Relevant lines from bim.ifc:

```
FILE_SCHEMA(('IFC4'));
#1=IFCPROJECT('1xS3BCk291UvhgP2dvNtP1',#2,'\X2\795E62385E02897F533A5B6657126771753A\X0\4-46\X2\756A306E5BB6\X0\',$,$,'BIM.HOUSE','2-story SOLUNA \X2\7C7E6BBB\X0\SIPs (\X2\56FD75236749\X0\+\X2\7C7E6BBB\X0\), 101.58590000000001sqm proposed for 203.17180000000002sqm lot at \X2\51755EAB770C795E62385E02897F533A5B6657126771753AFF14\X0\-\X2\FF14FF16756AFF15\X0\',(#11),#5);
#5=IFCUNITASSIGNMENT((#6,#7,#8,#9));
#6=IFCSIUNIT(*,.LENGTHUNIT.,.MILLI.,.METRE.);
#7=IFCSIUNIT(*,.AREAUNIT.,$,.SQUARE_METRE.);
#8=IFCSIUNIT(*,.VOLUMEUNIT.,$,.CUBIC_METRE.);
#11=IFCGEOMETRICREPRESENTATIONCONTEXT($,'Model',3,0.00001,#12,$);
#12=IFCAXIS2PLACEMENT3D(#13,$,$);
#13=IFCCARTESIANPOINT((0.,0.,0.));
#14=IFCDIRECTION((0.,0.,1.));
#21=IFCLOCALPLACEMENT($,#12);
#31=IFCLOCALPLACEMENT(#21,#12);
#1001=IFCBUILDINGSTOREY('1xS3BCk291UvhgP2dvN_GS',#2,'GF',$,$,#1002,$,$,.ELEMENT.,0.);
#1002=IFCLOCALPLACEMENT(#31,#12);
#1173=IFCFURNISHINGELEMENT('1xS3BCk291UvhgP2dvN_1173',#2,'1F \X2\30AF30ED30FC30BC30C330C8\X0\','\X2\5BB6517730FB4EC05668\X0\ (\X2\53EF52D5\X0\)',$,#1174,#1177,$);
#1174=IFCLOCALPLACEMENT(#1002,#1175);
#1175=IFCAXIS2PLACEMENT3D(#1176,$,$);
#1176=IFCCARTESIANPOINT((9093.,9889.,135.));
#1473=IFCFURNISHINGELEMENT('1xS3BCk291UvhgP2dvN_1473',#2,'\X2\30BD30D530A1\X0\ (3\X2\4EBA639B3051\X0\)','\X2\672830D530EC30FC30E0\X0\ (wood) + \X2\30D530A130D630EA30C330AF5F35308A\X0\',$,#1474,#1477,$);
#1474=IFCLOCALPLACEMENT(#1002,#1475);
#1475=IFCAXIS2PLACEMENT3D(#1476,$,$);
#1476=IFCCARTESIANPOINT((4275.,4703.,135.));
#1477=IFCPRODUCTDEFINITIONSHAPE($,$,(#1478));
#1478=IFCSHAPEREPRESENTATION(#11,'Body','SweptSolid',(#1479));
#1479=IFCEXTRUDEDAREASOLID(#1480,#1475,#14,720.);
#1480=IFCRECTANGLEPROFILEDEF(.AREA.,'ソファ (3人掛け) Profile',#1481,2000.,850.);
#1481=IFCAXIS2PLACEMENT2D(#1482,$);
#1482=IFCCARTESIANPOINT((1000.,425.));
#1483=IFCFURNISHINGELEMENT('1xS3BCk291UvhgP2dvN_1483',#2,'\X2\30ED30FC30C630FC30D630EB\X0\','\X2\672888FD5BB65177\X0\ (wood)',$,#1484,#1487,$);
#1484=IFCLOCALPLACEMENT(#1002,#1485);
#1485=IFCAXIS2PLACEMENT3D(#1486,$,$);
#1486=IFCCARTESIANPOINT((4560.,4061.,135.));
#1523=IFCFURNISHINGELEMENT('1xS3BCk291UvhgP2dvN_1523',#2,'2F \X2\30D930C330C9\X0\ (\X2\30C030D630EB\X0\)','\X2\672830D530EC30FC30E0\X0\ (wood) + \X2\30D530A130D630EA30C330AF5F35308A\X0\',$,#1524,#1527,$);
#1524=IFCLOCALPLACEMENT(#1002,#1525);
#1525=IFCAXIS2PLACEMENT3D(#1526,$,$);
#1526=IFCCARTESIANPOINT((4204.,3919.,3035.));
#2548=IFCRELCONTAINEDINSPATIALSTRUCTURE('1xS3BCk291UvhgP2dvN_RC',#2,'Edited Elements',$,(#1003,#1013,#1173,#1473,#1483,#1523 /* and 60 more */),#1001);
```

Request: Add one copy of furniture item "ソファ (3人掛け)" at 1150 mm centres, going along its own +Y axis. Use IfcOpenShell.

```python
import ifcopenshell
import ifcopenshell.api.geometry
import ifcopenshell.api.root
import ifcopenshell.util.element
import ifcopenshell.util.placement

model = ifcopenshell.open("bim.ifc")


def reuse_history(source, copy):
    """copy_class also copies each property set's owner history, people and application; keep the originals."""
    for rel in copy.IsDefinedBy:
        if rel.is_a("IfcRelDefinesByProperties") and (history := rel.RelatingPropertyDefinition.OwnerHistory):
            rel.RelatingPropertyDefinition.OwnerHistory = source.OwnerHistory
            ifcopenshell.util.element.remove_deep2(model, history)


source = model.by_guid("1xS3BCk291UvhgP2dvN_1473")
base = ifcopenshell.util.placement.get_local_placement(source.ObjectPlacement)
step = base[:3, 1] * 1150.0

for i in range(1, 2):
    copy = ifcopenshell.api.root.copy_class(model, product=source)
    copy.Representation = ifcopenshell.util.element.copy_deep(
        model, source.Representation, exclude=["IfcGeometricRepresentationContext", "IfcRepresentationMap"]
    )
    reuse_history(source, copy)
    matrix = base.copy()
    matrix[:3, 3] += i * step
    print("added at", matrix[:3, 3].round(3) + 0.0)
    ifcopenshell.api.geometry.edit_object_placement(model, product=copy, matrix=matrix, is_si=False)

model.write("bim_v2.ifc")
```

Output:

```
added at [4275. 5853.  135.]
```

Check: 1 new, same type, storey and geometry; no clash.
